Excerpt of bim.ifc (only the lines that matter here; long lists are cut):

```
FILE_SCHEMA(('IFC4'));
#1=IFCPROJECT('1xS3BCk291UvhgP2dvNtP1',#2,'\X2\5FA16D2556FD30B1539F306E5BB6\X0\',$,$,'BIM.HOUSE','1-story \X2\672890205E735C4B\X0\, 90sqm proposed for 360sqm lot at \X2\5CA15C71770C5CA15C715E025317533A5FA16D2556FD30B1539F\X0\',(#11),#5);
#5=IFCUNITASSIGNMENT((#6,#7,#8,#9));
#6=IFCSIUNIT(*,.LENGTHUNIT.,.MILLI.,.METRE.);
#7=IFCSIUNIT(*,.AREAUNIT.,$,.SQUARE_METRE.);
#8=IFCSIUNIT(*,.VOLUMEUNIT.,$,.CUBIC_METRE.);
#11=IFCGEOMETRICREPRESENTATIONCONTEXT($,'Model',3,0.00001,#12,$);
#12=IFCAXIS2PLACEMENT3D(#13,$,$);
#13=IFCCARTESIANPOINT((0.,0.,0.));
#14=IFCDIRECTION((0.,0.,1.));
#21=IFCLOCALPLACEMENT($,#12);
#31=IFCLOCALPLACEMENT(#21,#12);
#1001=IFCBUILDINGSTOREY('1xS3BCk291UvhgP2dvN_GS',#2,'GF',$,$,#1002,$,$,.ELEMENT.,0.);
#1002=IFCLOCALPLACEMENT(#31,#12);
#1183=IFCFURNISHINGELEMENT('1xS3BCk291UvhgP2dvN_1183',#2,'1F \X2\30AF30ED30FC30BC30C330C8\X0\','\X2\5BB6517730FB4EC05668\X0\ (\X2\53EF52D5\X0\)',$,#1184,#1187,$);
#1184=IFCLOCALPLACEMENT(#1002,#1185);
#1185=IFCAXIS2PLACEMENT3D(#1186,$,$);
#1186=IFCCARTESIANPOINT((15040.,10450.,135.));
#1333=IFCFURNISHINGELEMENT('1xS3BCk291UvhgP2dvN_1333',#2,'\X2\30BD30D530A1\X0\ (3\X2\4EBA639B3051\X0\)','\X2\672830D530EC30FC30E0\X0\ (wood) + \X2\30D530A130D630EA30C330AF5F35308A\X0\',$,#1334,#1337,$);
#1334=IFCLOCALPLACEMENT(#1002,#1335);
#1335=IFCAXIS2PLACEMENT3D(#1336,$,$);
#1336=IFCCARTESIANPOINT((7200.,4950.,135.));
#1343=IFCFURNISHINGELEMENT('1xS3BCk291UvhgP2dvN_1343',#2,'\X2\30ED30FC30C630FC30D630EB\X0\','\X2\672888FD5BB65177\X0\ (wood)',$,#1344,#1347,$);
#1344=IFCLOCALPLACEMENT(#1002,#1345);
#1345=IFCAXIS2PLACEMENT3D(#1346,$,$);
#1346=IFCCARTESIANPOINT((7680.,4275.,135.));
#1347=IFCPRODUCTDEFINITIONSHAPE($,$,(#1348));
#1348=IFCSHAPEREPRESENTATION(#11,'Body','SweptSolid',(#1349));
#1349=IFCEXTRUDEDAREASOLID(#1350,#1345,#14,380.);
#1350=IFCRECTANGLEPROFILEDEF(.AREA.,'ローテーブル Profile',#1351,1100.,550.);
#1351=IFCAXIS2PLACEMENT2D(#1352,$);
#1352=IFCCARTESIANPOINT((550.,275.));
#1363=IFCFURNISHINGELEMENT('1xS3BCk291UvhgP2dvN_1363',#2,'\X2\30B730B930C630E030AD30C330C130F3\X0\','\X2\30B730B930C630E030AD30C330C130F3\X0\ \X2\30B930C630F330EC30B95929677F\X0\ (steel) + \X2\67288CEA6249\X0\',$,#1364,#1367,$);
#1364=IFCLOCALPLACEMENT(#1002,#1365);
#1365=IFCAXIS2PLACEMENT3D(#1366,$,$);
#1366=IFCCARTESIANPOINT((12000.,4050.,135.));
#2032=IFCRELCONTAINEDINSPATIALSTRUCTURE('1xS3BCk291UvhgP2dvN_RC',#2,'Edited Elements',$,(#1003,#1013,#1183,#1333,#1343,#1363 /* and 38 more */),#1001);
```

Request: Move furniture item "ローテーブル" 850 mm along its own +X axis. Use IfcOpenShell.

```python
import ifcopenshell
import ifcopenshell.api.geometry
import ifcopenshell.util.placement

model = ifcopenshell.open("bim.ifc")

item = model.by_guid("1xS3BCk291UvhgP2dvN_1343")
matrix = ifcopenshell.util.placement.get_local_placement(item.ObjectPlacement)
matrix[:3, 3] += matrix[:3, 0] * 850.0
ifcopenshell.api.geometry.edit_object_placement(model, product=item, matrix=matrix, is_si=False)

print(ifcopenshell.util.placement.get_local_placement(item.ObjectPlacement).round(3) + 0.0)

model.write("bim_rev.ifc")
```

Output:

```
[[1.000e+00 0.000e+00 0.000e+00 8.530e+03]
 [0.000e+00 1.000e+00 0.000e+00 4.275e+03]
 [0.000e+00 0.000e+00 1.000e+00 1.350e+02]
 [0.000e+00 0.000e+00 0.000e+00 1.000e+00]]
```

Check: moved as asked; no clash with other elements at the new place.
